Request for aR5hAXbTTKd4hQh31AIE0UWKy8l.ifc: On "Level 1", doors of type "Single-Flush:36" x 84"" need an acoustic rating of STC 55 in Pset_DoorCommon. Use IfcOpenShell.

First a look at what the model holds.

```python
import ifcopenshell
import ifcopenshell.util.element

model = ifcopenshell.open("aR5hAXbTTKd4hQh31AIE0UWKy8l.ifc")
print(model.schema)
storey = next(s for s in model.by_type("IfcBuildingStorey") if s.Name == "Level 1")
doors = [e for e in ifcopenshell.util.element.get_decomposition(storey) if e.is_a("IfcDoor")]
seen = {}
for e in doors:
    element_type = ifcopenshell.util.element.get_type(e)
    key = (element_type.Name if element_type != e and element_type else None, ifcopenshell.util.element.get_pset(e, "Pset_DoorCommon", "AcousticRating"))
    seen[key] = seen.get(key, 0) + 1
for (name, value), count in sorted(seen.items(), key=str):
    print(count, "x", name, "|", value)
```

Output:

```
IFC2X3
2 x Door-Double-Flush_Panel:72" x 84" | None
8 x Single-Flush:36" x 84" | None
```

```python
import ifcopenshell
import ifcopenshell.api.pset
import ifcopenshell.util.element

model = ifcopenshell.open("aR5hAXbTTKd4hQh31AIE0UWKy8l.ifc")

storey = next(s for s in model.by_type("IfcBuildingStorey") if s.Name == "Level 1")
doors = [e for e in ifcopenshell.util.element.get_decomposition(storey) if e.is_a("IfcDoor")]

count = 0
for e in doors:
    element_type = ifcopenshell.util.element.get_type(e)
    if element_type in (None, e) or element_type.Name != 'Single-Flush:36" x 84"':
        continue
    # add_pset returns the element's existing set when there is one.
    pset = ifcopenshell.api.pset.add_pset(model, product=e, name="Pset_DoorCommon")
    ifcopenshell.api.pset.edit_pset(model, pset=pset, properties={"AcousticRating": "STC 55"})
    count += 1

print(count, "doors updated")

model.write("aR5hAXbTTKd4hQh31AIE0UWKy8l_v2.ifc")
```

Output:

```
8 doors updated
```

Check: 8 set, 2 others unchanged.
